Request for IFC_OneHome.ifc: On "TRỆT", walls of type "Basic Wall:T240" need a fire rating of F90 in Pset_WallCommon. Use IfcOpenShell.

First a look at what the model holds.

```python
import ifcopenshell
import ifcopenshell.util.element

model = ifcopenshell.open("IFC_OneHome.ifc")
print(model.schema)
storey = next(s for s in model.by_type("IfcBuildingStorey") if s.Name == "TRỆT")
walls = [e for e in ifcopenshell.util.element.get_decomposition(storey) if e.is_a("IfcWall")]
seen = {}
for e in walls:
    element_type = ifcopenshell.util.element.get_type(e)
    key = (element_type.Name if element_type != e and element_type else None, ifcopenshell.util.element.get_pset(e, "Pset_WallCommon", "FireRating"))
    seen[key] = seen.get(key, 0) + 1
for (name, value), count in sorted(seen.items(), key=str):
    print(count, "x", name, "|", value)
```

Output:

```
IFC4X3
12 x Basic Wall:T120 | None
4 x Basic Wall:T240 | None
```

```python
import ifcopenshell
import ifcopenshell.api.pset
import ifcopenshell.util.element

model = ifcopenshell.open("IFC_OneHome.ifc")

storey = next(s for s in model.by_type("IfcBuildingStorey") if s.Name == "TRỆT")
walls = [e for e in ifcopenshell.util.element.get_decomposition(storey) if e.is_a("IfcWall")]

count = 0
for e in walls:
    element_type = ifcopenshell.util.element.get_type(e)
    if element_type in (None, e) or element_type.Name != "Basic Wall:T240":
        continue
    # add_pset returns the element's existing set when there is one.
    pset = ifcopenshell.api.pset.add_pset(model, product=e, name="Pset_WallCommon")
    ifcopenshell.api.pset.edit_pset(model, pset=pset, properties={"FireRating": "F90"})
    count += 1

print(count, "walls updated")

model.write("IFC_OneHome_rev.ifc")
```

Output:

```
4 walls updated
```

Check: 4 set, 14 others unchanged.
